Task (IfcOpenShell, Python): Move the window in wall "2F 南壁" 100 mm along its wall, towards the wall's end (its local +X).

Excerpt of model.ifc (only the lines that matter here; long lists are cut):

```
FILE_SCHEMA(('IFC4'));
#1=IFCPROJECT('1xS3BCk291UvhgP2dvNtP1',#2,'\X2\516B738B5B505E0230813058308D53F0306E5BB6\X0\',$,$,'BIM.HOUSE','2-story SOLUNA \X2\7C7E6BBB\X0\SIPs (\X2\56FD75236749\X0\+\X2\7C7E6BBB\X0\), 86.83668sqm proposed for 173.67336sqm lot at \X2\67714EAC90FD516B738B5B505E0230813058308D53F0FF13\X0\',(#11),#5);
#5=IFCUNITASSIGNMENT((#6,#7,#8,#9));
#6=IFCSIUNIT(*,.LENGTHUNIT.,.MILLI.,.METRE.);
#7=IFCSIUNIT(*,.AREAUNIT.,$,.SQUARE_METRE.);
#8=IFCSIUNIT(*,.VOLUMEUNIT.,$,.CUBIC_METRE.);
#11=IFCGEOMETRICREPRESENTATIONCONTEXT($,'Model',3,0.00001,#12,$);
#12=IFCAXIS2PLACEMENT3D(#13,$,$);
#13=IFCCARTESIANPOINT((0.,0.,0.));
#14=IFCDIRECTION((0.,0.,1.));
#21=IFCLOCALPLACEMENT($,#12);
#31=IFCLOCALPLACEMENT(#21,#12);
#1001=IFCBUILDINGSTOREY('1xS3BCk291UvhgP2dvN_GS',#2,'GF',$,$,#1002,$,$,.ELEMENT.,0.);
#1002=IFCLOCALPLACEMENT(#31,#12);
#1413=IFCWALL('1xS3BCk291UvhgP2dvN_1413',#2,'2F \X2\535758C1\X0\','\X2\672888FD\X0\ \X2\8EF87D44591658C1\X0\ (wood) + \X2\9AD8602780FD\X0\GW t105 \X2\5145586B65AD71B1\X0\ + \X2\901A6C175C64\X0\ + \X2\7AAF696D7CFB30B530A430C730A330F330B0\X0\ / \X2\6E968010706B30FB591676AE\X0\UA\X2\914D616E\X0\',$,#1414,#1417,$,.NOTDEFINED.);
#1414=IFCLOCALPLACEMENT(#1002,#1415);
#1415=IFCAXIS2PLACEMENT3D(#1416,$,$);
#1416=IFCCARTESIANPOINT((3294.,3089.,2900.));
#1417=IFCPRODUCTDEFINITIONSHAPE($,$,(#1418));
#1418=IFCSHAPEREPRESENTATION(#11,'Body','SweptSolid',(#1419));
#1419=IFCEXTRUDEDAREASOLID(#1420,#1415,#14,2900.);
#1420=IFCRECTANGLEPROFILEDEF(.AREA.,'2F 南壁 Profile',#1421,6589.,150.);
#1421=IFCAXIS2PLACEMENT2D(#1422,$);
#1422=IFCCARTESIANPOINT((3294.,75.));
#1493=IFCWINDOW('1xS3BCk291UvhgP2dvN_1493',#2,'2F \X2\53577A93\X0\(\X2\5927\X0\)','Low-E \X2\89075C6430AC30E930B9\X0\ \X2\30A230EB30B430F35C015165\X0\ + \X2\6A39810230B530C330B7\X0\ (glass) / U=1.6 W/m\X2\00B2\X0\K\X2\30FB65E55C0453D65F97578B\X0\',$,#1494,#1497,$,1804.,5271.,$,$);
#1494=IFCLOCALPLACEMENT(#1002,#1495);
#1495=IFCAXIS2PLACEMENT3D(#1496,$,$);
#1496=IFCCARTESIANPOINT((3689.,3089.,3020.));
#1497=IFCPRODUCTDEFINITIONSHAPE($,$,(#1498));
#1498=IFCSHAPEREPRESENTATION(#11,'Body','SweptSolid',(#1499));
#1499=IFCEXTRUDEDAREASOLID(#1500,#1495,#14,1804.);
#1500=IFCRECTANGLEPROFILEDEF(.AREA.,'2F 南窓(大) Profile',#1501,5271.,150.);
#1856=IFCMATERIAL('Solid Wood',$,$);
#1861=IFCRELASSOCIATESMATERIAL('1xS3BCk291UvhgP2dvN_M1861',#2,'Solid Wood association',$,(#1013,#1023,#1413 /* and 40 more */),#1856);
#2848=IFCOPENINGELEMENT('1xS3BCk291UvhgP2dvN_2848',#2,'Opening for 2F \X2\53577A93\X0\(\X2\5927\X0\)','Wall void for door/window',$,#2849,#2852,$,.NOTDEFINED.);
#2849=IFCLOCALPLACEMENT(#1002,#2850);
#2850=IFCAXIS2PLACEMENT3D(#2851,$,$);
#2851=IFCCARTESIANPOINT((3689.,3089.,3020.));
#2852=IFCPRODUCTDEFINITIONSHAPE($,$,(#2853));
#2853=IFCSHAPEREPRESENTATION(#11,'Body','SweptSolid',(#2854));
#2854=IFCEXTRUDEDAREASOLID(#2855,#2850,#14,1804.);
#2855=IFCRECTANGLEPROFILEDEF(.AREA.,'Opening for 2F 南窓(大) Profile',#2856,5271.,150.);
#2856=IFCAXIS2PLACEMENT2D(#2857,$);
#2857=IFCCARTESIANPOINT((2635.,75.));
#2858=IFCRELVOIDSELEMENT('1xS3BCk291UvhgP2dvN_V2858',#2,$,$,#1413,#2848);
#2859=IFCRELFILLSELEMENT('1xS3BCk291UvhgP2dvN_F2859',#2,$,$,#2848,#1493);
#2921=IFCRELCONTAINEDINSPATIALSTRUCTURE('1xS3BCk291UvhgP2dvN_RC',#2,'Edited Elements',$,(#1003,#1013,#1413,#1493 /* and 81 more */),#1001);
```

```python
import ifcopenshell
import ifcopenshell.api.geometry
import ifcopenshell.util.placement

model = ifcopenshell.open("model.ifc")

window = model.by_guid("1xS3BCk291UvhgP2dvN_1493")
opening = window.FillsVoids[0].RelatingOpeningElement
wall = opening.VoidsElements[0].RelatingBuildingElement

wall_matrix = ifcopenshell.util.placement.get_local_placement(wall.ObjectPlacement)
shift = wall_matrix[:3, 0] * 100.0
before = ifcopenshell.util.placement.get_local_placement(window.ObjectPlacement)[:3, 3].copy()

# The window is not placed relative to its opening, so move both.
for product in (opening, window):
    matrix = ifcopenshell.util.placement.get_local_placement(product.ObjectPlacement)
    matrix[:3, 3] += shift
    ifcopenshell.api.geometry.edit_object_placement(model, product=product, matrix=matrix, is_si=False)

after = ifcopenshell.util.placement.get_local_placement(window.ObjectPlacement)[:3, 3]
print("window moved by", (after - before).round(3) + 0.0)

model.write("model_v2.ifc")
```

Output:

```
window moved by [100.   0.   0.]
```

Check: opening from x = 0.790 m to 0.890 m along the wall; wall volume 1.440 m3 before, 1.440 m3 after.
